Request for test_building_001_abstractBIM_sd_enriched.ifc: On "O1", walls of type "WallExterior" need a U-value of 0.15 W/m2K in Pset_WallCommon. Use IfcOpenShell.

First a look at what the model holds.

```python
import ifcopenshell
import ifcopenshell.util.element

model = ifcopenshell.open("test_building_001_abstractBIM_sd_enriched.ifc")
print(model.schema)
storey = next(s for s in model.by_type("IfcBuildingStorey") if s.Name == "O1")
walls = [e for e in ifcopenshell.util.element.get_decomposition(storey) if e.is_a("IfcWall")]
seen = {}
for e in walls:
    element_type = ifcopenshell.util.element.get_type(e)
    key = (element_type.Name if element_type != e and element_type else None, ifcopenshell.util.element.get_pset(e, "Pset_WallCommon", "ThermalTransmittance"))
    seen[key] = seen.get(key, 0) + 1
for (name, value), count in sorted(seen.items(), key=str):
    print(count, "x", name, "|", value)
```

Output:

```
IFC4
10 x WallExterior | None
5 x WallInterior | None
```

```python
import ifcopenshell
import ifcopenshell.api.pset
import ifcopenshell.util.element

model = ifcopenshell.open("test_building_001_abstractBIM_sd_enriched.ifc")

storey = next(s for s in model.by_type("IfcBuildingStorey") if s.Name == "O1")
walls = [e for e in ifcopenshell.util.element.get_decomposition(storey) if e.is_a("IfcWall")]

count = 0
for e in walls:
    element_type = ifcopenshell.util.element.get_type(e)
    if element_type in (None, e) or element_type.Name != "WallExterior":
        continue
    # add_pset returns the element's existing set when there is one.
    pset = ifcopenshell.api.pset.add_pset(model, product=e, name="Pset_WallCommon")
    ifcopenshell.api.pset.edit_pset(model, pset=pset, properties={"ThermalTransmittance": 0.15})
    count += 1

print(count, "walls updated")

model.write("test_building_001_abstractBIM_sd_enriched_v2.ifc")
```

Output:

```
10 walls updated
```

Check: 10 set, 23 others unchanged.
